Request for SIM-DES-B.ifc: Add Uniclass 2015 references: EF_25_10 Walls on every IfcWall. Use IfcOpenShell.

First a look at what the model holds.

```python
import ifcopenshell

model = ifcopenshell.open("SIM-DES-B.ifc")
print(model.schema)
print("classifications:", [c.Name for c in model.by_type("IfcClassification")])
for ifc_class in ("IfcDoor", "IfcRoof", "IfcStair", "IfcWall", "IfcWindow"):
    print(ifc_class, len(model.by_type(ifc_class)))
```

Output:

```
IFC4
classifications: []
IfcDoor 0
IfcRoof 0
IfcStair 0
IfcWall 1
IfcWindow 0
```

```python
import ifcopenshell
import ifcopenshell.api.classification

model = ifcopenshell.open("SIM-DES-B.ifc")

system = ifcopenshell.api.classification.add_classification(model, classification="Uniclass 2015")

codes = {
    "IfcWall": ("EF_25_10", "Walls"),
}
for ifc_class, (code, name) in codes.items():
    products = model.by_type(ifc_class)
    ifcopenshell.api.classification.add_reference(
        model, products=products, classification=system, identification=code, name=name
    )
    print(code, len(products))

model.write("SIM-DES-B-out.ifc")
```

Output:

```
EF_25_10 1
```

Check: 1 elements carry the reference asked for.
